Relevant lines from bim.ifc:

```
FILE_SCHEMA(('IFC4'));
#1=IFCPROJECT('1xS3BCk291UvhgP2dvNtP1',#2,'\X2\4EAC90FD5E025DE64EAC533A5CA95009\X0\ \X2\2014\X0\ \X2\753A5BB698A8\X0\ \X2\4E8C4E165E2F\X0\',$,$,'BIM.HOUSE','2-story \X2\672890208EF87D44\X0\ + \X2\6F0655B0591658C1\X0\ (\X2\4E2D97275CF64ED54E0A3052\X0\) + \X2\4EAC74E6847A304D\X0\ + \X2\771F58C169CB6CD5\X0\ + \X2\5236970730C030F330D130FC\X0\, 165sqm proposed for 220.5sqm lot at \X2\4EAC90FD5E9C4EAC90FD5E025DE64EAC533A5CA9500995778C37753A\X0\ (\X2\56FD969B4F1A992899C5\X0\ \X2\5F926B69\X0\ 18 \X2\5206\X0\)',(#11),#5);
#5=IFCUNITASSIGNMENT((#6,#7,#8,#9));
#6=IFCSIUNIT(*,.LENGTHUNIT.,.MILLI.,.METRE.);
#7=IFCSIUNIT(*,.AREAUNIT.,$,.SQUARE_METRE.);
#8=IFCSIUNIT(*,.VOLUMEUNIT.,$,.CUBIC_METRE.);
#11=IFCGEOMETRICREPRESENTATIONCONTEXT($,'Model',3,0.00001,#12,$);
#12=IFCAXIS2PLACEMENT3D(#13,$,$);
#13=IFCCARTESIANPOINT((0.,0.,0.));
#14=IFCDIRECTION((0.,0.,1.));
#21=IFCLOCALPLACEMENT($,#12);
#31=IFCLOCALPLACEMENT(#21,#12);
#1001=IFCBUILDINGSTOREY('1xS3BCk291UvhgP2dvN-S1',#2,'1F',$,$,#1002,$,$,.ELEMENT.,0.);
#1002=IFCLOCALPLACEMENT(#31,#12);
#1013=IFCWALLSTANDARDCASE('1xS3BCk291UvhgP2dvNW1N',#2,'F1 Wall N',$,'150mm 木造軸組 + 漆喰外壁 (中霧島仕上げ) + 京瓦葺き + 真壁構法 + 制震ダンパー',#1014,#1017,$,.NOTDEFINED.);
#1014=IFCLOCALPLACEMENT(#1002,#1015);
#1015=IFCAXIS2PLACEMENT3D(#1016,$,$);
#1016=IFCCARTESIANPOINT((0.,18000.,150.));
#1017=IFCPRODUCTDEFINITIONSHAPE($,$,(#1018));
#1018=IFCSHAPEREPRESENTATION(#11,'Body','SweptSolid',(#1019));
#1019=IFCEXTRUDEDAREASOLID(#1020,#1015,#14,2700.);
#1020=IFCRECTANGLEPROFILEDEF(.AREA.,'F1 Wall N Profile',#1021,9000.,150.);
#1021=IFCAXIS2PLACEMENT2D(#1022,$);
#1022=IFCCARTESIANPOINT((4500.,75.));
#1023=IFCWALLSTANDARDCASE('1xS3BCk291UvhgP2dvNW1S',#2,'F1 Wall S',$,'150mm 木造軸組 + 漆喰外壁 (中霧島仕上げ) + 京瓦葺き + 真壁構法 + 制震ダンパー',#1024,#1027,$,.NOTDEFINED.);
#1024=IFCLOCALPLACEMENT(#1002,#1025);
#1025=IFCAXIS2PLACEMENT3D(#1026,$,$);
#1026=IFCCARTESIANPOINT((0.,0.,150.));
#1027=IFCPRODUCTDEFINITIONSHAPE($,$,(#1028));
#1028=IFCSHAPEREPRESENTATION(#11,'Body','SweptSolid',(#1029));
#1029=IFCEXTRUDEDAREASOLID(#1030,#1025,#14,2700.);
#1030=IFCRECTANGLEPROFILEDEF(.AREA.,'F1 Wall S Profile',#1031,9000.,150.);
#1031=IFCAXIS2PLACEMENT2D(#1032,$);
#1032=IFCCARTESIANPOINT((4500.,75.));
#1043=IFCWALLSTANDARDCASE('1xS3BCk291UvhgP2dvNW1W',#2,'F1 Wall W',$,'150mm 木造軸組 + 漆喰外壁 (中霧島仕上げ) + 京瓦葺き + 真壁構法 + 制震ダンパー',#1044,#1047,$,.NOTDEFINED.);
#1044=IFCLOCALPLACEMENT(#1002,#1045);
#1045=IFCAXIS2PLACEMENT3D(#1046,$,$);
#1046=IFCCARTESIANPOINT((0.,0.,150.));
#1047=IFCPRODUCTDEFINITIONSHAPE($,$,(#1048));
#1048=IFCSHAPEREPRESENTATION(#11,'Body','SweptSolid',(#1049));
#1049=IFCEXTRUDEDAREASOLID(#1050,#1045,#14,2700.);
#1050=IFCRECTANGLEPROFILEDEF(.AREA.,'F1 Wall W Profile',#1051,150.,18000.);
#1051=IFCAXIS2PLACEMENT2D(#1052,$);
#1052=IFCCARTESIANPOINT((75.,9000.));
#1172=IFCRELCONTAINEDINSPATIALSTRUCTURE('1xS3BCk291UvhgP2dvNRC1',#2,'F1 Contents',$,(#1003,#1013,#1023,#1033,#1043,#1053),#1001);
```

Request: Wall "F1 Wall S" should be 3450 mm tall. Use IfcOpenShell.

```python
import ifcopenshell
import ifcopenshell.geom
import ifcopenshell.util.shape
import ifcopenshell.util.unit

model = ifcopenshell.open("bim.ifc")
unit_scale = ifcopenshell.util.unit.calculate_unit_scale(model)
settings = ifcopenshell.geom.settings()


def volume(element):
    """Net volume in cubic metres, openings subtracted."""
    shape = ifcopenshell.geom.create_shape(settings, element)
    return ifcopenshell.util.shape.get_volume(shape.geometry)


wall = model.by_guid("1xS3BCk291UvhgP2dvNW1S")
before = volume(wall)

body = next(r for r in wall.Representation.Representations if r.RepresentationIdentifier == "Body")
solid = body.Items[0]
old_height = solid.Depth
solid.Depth = 3.45 / unit_scale
after = volume(wall)

print(f"height {old_height:g} -> {solid.Depth:g}, volume {before:.3f} -> {after:.3f} m3")

model.write("bim_edited.ifc")
```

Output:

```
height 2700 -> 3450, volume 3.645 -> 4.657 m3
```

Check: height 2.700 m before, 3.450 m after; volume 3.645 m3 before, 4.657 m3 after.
